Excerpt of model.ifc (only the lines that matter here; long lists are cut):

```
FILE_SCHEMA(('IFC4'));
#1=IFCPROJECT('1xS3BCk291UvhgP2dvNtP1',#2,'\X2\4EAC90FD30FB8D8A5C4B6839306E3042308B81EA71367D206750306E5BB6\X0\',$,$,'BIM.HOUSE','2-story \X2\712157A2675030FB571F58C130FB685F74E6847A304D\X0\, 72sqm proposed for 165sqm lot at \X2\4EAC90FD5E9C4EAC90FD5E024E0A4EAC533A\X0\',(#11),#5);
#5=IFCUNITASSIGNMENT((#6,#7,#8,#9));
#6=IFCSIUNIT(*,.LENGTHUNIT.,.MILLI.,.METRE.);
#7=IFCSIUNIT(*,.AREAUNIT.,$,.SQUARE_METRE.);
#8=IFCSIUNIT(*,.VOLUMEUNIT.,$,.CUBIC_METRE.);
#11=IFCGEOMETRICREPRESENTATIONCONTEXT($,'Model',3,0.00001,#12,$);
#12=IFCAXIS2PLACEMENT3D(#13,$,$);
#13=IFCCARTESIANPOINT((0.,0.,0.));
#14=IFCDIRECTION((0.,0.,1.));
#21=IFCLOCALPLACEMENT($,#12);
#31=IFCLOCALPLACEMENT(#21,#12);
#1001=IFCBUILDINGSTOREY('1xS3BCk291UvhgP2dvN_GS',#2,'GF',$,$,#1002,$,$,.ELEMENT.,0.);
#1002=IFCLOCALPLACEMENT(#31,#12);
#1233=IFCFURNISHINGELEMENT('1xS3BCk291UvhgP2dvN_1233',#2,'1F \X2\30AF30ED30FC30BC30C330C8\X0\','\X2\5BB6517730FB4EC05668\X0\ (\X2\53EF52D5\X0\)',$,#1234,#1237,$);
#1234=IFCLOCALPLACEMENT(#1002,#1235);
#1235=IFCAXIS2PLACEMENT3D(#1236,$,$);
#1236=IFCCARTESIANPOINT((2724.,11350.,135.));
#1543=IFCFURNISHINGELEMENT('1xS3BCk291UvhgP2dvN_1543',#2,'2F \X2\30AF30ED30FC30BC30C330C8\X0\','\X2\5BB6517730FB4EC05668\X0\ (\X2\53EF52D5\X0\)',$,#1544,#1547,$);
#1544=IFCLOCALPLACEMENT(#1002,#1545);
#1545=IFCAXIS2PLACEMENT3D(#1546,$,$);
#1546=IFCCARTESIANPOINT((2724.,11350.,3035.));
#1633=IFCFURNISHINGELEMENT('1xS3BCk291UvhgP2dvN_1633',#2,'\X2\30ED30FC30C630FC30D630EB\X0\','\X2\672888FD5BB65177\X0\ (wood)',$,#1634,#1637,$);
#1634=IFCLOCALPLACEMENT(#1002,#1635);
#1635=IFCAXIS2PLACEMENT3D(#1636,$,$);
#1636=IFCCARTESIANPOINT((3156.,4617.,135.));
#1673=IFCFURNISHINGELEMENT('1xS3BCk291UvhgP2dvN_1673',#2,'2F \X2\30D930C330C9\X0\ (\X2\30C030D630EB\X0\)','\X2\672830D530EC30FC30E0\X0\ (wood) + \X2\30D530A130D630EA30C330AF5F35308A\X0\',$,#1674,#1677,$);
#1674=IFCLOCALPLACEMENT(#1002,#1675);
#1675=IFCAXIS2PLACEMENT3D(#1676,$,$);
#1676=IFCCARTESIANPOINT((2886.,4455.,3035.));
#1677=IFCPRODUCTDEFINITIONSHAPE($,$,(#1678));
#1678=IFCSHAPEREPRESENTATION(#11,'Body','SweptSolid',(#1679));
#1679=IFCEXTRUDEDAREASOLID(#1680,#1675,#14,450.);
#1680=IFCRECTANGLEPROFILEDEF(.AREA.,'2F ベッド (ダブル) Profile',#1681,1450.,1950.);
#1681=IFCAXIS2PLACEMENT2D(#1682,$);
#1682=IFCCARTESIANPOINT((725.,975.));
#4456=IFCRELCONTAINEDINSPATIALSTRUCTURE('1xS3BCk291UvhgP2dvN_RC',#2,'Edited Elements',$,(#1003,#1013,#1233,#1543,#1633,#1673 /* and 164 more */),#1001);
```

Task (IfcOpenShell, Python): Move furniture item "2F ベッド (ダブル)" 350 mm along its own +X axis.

```python
import ifcopenshell
import ifcopenshell.api.geometry
import ifcopenshell.util.placement
import ifcopenshell.util.unit

model = ifcopenshell.open("model.ifc")
unit_scale = ifcopenshell.util.unit.calculate_unit_scale(model)

item = model.by_id(1673)
matrix = ifcopenshell.util.placement.get_local_placement(item.ObjectPlacement)
matrix[:3, 3] += matrix[:3, 0] * 0.35 / unit_scale
ifcopenshell.api.geometry.edit_object_placement(model, product=item, matrix=matrix, is_si=False)

print(ifcopenshell.util.placement.get_local_placement(item.ObjectPlacement).round(3) + 0.0)

model.write("model_updated.ifc")
```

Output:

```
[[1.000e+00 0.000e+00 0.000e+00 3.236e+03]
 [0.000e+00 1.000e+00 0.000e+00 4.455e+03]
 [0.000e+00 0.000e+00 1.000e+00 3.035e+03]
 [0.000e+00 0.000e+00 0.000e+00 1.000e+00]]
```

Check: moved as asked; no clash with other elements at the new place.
